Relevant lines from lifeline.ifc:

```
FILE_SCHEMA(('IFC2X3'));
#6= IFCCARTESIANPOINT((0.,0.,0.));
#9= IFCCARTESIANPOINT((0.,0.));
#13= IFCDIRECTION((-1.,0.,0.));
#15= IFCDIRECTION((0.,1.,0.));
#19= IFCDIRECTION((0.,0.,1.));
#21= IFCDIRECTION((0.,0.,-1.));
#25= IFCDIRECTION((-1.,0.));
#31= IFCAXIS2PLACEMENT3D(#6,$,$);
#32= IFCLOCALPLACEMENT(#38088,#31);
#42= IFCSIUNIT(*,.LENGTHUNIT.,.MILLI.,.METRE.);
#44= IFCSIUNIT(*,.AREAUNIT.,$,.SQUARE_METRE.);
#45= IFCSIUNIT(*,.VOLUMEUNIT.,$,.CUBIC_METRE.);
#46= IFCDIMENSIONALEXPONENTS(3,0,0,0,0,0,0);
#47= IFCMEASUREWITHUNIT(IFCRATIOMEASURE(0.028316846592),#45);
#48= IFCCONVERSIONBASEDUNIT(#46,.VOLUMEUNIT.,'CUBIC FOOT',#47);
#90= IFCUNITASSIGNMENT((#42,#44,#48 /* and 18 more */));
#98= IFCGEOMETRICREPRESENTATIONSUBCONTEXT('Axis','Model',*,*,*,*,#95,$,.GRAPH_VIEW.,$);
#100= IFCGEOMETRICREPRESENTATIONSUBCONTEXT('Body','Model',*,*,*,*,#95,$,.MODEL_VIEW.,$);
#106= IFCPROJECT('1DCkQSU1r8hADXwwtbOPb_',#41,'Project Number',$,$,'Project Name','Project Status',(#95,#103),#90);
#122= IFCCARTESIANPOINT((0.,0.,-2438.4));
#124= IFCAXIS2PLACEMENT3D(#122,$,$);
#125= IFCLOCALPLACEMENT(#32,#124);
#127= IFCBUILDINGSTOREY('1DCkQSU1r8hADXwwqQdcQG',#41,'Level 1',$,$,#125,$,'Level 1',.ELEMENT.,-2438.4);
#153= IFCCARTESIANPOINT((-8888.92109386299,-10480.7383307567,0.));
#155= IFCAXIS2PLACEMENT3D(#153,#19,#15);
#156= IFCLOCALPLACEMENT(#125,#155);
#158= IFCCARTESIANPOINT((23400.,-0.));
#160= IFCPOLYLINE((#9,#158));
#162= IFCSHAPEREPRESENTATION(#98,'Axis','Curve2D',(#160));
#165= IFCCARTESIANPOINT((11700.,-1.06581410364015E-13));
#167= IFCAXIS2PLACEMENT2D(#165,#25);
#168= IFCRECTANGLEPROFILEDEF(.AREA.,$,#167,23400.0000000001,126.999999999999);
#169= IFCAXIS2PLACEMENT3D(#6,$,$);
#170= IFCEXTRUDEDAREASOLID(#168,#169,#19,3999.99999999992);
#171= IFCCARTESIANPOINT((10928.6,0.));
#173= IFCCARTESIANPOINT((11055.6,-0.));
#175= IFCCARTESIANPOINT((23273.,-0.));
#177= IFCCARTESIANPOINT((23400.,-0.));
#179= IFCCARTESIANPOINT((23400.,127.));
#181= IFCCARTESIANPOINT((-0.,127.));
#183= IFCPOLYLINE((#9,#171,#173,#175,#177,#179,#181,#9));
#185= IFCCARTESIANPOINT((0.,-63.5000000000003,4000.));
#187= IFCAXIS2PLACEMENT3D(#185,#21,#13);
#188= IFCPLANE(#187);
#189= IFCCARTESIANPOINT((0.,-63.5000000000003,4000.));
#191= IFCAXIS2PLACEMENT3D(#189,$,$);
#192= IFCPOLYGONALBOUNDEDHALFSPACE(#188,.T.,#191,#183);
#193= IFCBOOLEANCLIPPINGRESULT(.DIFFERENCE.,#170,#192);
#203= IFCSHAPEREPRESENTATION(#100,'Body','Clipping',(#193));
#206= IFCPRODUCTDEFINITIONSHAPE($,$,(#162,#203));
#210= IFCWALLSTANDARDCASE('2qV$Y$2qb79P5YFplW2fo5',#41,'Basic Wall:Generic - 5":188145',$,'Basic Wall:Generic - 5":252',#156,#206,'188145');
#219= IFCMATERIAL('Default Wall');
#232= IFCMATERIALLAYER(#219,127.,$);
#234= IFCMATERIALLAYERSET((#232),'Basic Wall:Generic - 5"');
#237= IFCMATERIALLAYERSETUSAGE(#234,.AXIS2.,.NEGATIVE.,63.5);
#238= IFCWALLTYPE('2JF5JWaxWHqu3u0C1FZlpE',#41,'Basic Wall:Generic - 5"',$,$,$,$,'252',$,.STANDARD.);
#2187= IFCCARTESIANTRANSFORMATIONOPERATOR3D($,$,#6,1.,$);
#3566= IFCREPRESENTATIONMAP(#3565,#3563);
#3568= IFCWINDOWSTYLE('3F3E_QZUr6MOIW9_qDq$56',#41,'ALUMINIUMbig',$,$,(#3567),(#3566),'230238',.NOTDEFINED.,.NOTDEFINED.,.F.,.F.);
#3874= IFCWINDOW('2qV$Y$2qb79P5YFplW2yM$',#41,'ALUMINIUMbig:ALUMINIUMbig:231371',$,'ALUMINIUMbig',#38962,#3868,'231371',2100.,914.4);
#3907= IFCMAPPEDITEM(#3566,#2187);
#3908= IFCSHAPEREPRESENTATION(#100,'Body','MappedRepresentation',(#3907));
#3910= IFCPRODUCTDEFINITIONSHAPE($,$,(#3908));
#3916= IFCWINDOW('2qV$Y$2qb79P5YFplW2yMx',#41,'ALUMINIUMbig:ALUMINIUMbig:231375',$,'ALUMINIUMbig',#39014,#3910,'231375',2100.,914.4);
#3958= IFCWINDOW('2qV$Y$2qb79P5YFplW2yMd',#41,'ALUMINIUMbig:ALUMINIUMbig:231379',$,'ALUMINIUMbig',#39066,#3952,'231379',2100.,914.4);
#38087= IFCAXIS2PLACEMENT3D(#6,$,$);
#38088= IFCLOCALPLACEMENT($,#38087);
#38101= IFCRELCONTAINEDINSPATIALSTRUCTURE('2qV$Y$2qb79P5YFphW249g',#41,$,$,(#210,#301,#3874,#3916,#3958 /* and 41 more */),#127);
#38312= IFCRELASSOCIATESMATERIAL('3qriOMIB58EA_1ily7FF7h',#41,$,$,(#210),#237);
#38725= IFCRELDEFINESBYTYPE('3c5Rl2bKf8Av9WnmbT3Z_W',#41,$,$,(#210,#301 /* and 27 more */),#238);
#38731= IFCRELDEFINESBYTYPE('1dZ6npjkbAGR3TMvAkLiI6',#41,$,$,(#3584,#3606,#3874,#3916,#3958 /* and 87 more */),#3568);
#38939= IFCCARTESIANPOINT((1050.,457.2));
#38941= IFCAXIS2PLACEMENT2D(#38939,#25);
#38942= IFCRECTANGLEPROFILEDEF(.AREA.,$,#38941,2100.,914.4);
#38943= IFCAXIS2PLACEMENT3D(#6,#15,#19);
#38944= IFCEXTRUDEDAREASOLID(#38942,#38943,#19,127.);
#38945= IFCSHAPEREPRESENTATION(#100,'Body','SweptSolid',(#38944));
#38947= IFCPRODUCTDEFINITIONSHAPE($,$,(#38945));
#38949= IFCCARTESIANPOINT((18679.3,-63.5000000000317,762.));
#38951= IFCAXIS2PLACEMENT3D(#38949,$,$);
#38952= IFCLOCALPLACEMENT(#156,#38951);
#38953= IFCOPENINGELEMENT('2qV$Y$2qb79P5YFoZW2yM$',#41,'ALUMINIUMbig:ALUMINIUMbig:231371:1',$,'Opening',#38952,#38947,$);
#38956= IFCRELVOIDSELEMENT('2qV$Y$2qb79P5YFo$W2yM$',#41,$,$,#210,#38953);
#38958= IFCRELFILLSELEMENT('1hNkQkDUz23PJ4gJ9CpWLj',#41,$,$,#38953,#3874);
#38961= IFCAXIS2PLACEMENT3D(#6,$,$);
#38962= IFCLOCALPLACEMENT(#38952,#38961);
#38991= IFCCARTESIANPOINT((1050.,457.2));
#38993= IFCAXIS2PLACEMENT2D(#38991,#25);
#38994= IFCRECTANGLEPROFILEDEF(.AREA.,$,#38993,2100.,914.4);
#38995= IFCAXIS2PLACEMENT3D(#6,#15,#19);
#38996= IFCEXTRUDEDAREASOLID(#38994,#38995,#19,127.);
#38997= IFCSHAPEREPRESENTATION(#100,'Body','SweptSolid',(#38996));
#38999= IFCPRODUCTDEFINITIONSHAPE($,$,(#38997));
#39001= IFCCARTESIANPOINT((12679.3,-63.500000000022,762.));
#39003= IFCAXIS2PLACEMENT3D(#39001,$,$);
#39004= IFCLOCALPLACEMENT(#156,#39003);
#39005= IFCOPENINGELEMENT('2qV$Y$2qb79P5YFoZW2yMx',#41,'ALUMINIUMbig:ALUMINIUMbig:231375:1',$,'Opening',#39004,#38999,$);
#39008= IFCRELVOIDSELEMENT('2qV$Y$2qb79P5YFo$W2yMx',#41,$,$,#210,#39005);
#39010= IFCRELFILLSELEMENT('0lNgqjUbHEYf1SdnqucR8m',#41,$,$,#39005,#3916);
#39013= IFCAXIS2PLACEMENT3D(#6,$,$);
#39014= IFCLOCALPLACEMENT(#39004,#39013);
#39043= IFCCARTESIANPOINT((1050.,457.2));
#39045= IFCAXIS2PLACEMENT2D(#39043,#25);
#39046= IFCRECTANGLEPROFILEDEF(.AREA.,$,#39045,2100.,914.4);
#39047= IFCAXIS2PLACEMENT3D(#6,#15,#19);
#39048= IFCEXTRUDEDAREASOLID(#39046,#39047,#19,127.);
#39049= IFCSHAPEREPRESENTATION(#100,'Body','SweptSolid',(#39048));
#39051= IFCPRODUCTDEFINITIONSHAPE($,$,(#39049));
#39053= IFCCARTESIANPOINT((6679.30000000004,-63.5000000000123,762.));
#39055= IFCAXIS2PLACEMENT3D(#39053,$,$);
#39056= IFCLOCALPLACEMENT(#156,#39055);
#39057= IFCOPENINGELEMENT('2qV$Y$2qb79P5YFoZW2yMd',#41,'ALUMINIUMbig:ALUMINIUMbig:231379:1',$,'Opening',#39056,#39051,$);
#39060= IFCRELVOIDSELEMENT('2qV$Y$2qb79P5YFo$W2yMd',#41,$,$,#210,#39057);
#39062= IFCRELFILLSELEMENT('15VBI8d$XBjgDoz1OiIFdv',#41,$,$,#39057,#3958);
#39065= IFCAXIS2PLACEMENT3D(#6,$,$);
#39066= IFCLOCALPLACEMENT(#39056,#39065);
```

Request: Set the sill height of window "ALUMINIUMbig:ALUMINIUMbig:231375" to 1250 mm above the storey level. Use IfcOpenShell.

```python
import numpy as np
import ifcopenshell
import ifcopenshell.api.geometry
import ifcopenshell.geom
import ifcopenshell.util.element
import ifcopenshell.util.placement
import ifcopenshell.util.shape
import ifcopenshell.util.unit

model = ifcopenshell.open("lifeline.ifc")
unit_scale = ifcopenshell.util.unit.calculate_unit_scale(model)

window = model.by_id(3916)
opening = window.FillsVoids[0].RelatingOpeningElement
storey = ifcopenshell.util.element.get_container(window, ifc_class="IfcBuildingStorey")
level = ifcopenshell.util.placement.get_local_placement(storey.ObjectPlacement)[2, 3]

# The opening's origin need not be at the sill, so measure its lowest point.
shape = ifcopenshell.geom.create_shape(ifcopenshell.geom.settings(), opening)
bottom = ifcopenshell.util.shape.get_shape_bottom_elevation(shape, shape.geometry) / unit_scale
dz = level + 1250.0 - bottom

shift = np.array([0.0, 0.0, dz])
# The window is placed relative to its opening, so it follows when the opening moves.
matrix = ifcopenshell.util.placement.get_local_placement(opening.ObjectPlacement)
matrix[:3, 3] += shift
ifcopenshell.api.geometry.edit_object_placement(
    model, product=opening, matrix=matrix, is_si=False, should_transform_children=True
)

print(f"moved by {dz * unit_scale:+.3f} m")

model.write("lifeline_rev.ifc")
```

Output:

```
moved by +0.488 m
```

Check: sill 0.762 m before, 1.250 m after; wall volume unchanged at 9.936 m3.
